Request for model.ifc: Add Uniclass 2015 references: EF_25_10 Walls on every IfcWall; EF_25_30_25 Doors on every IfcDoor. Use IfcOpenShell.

First a look at what the model holds.

```python
import ifcopenshell

model = ifcopenshell.open("model.ifc")
print(model.schema)
print("classifications:", [c.Name for c in model.by_type("IfcClassification")])
for ifc_class in ("IfcDoor", "IfcRoof", "IfcStair", "IfcWall", "IfcWindow"):
    print(ifc_class, len(model.by_type(ifc_class)))
```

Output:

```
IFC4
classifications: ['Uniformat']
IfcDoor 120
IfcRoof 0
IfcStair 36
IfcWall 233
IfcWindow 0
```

```python
import ifcopenshell
import ifcopenshell.api.classification

model = ifcopenshell.open("model.ifc")

system = ifcopenshell.api.classification.add_classification(model, classification="Uniclass 2015")

codes = {
    "IfcWall": ("EF_25_10", "Walls"),
    "IfcDoor": ("EF_25_30_25", "Doors"),
}
for ifc_class, (code, name) in codes.items():
    products = model.by_type(ifc_class)
    ifcopenshell.api.classification.add_reference(
        model, products=products, classification=system, identification=code, name=name
    )
    print(code, len(products))

model.write("model_edited.ifc")
```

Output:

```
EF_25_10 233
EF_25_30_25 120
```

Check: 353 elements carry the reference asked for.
